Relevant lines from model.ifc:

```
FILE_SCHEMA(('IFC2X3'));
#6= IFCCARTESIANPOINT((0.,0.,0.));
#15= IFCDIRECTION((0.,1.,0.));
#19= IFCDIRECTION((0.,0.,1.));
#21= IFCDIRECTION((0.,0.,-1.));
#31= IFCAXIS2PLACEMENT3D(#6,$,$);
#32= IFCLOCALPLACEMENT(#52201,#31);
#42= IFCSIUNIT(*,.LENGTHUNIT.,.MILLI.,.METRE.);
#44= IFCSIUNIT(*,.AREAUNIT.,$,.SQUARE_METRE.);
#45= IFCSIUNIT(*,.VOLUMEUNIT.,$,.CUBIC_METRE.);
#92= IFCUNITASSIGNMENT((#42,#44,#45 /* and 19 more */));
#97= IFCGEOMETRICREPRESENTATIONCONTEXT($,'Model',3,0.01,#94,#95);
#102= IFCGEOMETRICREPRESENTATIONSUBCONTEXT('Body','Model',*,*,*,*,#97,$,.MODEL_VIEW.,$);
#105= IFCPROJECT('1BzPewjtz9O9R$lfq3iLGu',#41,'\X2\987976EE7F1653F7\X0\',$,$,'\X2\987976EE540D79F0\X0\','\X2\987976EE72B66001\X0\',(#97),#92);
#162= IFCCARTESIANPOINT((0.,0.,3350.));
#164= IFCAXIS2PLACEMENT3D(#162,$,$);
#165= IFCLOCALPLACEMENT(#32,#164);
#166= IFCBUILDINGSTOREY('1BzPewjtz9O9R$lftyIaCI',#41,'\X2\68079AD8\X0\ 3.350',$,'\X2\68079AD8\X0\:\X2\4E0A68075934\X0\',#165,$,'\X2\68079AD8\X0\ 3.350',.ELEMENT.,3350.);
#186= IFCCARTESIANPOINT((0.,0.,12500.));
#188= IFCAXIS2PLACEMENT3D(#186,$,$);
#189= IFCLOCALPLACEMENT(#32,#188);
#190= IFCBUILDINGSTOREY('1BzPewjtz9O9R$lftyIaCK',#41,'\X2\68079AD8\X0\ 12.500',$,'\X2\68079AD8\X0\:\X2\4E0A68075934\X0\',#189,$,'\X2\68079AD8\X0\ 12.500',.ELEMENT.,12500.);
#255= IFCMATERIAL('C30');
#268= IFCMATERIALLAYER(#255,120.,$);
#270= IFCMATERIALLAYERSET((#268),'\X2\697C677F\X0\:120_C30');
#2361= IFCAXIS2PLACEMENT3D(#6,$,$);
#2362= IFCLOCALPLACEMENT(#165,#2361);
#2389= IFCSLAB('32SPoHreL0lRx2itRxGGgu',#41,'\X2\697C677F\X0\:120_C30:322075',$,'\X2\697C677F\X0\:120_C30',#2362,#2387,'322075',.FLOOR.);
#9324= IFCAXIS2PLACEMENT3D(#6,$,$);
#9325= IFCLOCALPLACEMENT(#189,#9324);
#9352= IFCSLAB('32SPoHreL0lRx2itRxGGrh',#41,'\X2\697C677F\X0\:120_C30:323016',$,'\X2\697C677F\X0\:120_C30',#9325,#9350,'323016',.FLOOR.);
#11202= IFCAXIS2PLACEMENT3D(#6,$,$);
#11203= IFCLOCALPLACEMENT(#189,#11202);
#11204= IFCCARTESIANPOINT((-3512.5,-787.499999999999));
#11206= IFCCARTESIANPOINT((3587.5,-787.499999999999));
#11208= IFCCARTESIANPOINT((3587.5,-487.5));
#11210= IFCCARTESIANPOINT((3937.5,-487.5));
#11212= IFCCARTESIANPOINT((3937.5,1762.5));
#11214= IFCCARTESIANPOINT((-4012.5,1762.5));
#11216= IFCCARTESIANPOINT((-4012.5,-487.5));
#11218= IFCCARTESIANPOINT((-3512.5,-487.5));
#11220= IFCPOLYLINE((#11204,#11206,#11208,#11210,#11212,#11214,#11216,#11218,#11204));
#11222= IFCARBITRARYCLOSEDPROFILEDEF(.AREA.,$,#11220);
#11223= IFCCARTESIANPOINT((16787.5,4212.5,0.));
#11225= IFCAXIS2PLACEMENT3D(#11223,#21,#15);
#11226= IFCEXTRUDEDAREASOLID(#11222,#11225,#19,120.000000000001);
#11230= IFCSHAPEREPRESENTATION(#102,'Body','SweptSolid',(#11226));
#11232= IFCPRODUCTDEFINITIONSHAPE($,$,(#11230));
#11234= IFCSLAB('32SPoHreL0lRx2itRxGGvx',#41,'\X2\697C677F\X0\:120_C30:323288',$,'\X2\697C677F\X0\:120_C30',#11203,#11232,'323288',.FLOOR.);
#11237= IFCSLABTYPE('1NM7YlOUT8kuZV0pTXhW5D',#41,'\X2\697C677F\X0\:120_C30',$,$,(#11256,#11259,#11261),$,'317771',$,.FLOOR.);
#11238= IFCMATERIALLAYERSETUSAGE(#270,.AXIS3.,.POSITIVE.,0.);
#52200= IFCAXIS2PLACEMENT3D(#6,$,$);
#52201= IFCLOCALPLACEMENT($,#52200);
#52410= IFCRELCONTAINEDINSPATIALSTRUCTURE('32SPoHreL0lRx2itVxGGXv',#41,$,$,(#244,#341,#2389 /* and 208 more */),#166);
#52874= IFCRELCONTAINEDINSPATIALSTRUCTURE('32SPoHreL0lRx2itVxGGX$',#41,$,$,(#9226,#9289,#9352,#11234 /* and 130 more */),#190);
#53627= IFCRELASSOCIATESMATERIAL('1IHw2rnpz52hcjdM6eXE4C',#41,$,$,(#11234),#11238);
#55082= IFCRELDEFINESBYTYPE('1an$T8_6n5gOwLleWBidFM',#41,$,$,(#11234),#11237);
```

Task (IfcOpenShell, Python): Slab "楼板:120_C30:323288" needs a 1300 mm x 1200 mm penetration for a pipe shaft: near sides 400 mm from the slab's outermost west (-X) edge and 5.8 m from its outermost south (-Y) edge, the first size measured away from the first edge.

```python
import numpy as np
import ifcopenshell
import ifcopenshell.api.feature
import ifcopenshell.api.geometry
import ifcopenshell.api.root
import ifcopenshell.geom
import ifcopenshell.util.placement
import ifcopenshell.util.representation
import ifcopenshell.util.shape
import ifcopenshell.util.unit

model = ifcopenshell.open("model.ifc")
unit_scale = ifcopenshell.util.unit.calculate_unit_scale(model)
settings = ifcopenshell.geom.settings()


def volume(element):
    """Net volume in cubic metres, openings subtracted."""
    shape = ifcopenshell.geom.create_shape(settings, element)
    return ifcopenshell.util.shape.get_volume(shape.geometry)


slab = model.by_guid("32SPoHreL0lRx2itRxGGvx")
before = volume(slab)

# Extent in the slab's own axes, in metres. The edges named are its -X and -Y sides.
slab_shape = ifcopenshell.geom.create_shape(settings, slab)
vertices = ifcopenshell.util.shape.get_vertices(slab_shape.geometry)
x_min, y_min, bottom = vertices.min(axis=0)
top = vertices[:, 2].max()

opening = ifcopenshell.api.root.create_entity(model, ifc_class="IfcOpeningElement", name="Pipe shaft opening")
context = ifcopenshell.util.representation.get_context(model, "Model", "Body", "MODEL_VIEW")
width, depth = 1.3, 1.2
outline = [(0.0, 0.0), (width, 0.0), (width, depth), (0.0, depth), (0.0, 0.0)]
# Overshoot both faces by 50 mm so the cut is clean.
shape = ifcopenshell.api.geometry.add_slab_representation(
    model, context=context, depth=top - bottom + 0.1, polyline=outline
)
ifcopenshell.api.geometry.assign_representation(model, product=opening, representation=shape)

matrix = ifcopenshell.util.placement.get_local_placement(slab.ObjectPlacement)
matrix[:, 3] = matrix @ np.append(np.array([x_min + 0.4, y_min + 5.8, bottom - 0.05]) / unit_scale, 1.0)
ifcopenshell.api.geometry.edit_object_placement(model, product=opening, matrix=matrix, is_si=False)
ifcopenshell.api.feature.add_feature(model, feature=opening, element=slab)

after = volume(slab)

print(f"slab volume {before:.3f} -> {after:.3f} m3")

model.write("model_rev.ifc")
```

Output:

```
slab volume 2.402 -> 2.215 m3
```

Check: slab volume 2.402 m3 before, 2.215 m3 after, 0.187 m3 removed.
